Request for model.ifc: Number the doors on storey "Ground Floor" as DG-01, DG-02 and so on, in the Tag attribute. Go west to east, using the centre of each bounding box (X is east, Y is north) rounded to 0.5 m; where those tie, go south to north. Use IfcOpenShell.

First a look at what the model holds.

```python
import ifcopenshell
import ifcopenshell.util.element
import ifcopenshell.util.placement

model = ifcopenshell.open("model.ifc")
print(model.schema)
storey = next(s for s in model.by_type("IfcBuildingStorey") if s.Name == "Ground Floor")
doors = [e for e in ifcopenshell.util.element.get_decomposition(storey) if e.is_a("IfcDoor")]
for e in sorted(doors, key=lambda e: e.id()):
    origin = ifcopenshell.util.placement.get_local_placement(e.ObjectPlacement)[:3, 3]
    print(e.id(), e.Tag, e.Name, origin.round(2) + 0.0, sep=" | ")
```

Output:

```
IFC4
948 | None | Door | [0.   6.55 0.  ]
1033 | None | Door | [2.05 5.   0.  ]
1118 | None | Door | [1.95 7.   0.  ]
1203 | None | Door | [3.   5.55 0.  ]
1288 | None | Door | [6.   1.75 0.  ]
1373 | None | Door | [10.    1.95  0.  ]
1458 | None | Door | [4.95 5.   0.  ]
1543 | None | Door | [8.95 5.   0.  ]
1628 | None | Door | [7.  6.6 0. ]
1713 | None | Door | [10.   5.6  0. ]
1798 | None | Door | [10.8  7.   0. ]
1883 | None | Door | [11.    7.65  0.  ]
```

```python
import ifcopenshell
import ifcopenshell.geom
import ifcopenshell.util.element
import ifcopenshell.util.shape

model = ifcopenshell.open("model.ifc")
settings = ifcopenshell.geom.settings()
settings.set("use-world-coords", True)


def centre(element):
    shape = ifcopenshell.geom.create_shape(settings, element)
    return ifcopenshell.util.shape.get_bbox_centroid(shape.geometry)


storey = next(s for s in model.by_type("IfcBuildingStorey") if s.Name == "Ground Floor")
doors = [e for e in ifcopenshell.util.element.get_decomposition(storey) if e.is_a("IfcDoor")]

# Insertion points can sit at a corner or the storey origin, so sort by the geometry (in metres).
centres = {e: centre(e) for e in doors}
doors.sort(key=lambda e: (round(centres[e][0] / 0.5), centres[e][1]))

for i, e in enumerate(doors, start=1):
    number = f"DG-{i:02d}"
    e.Tag = number
    print(e.id(), number)

model.write("model_updated.ifc")
```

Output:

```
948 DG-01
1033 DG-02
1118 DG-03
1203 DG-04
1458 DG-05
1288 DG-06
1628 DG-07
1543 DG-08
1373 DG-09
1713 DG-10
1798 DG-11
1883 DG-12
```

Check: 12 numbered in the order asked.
